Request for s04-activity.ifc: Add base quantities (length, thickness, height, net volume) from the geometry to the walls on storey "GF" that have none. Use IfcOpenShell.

First a look at what the model holds.

```python
import ifcopenshell
import ifcopenshell.util.element
import ifcopenshell.util.unit

model = ifcopenshell.open("s04-activity.ifc")
print(model.schema)
for unit_type in ("LENGTHUNIT", "AREAUNIT", "VOLUMEUNIT"):
    print(unit_type, ifcopenshell.util.unit.calculate_unit_scale(model, unit_type))
storey = next(s for s in model.by_type("IfcBuildingStorey") if s.Name == "GF")
walls = [e for e in ifcopenshell.util.element.get_decomposition(storey) if e.is_a("IfcWall")]
for e in sorted(walls, key=lambda e: e.id()):
    print(e.id(), e.is_a(), e.Name, list(ifcopenshell.util.element.get_psets(e, qtos_only=True)), sep=" | ")
```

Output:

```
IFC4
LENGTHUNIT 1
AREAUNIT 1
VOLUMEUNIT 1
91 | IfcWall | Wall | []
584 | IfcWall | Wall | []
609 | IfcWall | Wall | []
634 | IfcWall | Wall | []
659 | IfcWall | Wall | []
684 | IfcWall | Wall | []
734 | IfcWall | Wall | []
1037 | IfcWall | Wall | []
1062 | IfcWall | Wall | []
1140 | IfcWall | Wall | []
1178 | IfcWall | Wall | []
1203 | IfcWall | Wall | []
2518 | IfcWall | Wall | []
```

```python
import ifcopenshell
import ifcopenshell.api.pset
import ifcopenshell.geom
import ifcopenshell.util.element
import ifcopenshell.util.shape
import ifcopenshell.util.unit

model = ifcopenshell.open("s04-activity.ifc")
unit_scale = ifcopenshell.util.unit.calculate_unit_scale(model)
volume_scale = ifcopenshell.util.unit.calculate_unit_scale(model, "VOLUMEUNIT")
settings = ifcopenshell.geom.settings()

storey = next(s for s in model.by_type("IfcBuildingStorey") if s.Name == "GF")
walls = [e for e in ifcopenshell.util.element.get_decomposition(storey) if e.is_a("IfcWall")]

for e in sorted(walls, key=lambda e: e.id()):
    if ifcopenshell.util.element.get_psets(e, qtos_only=True, should_inherit=False):
        continue
    # Geometry comes back in metres, in the element's own axes.
    shape = ifcopenshell.geom.create_shape(settings, e)
    values = {
        "Length": ifcopenshell.util.shape.get_x(shape.geometry) / unit_scale,
        "Width": ifcopenshell.util.shape.get_y(shape.geometry) / unit_scale,
        "Height": ifcopenshell.util.shape.get_z(shape.geometry) / unit_scale,
        "NetVolume": ifcopenshell.util.shape.get_volume(shape.geometry) / volume_scale,
    }
    qto = ifcopenshell.api.pset.add_qto(model, product=e, name="Qto_WallBaseQuantities")
    ifcopenshell.api.pset.edit_qto(model, qto=qto, properties=values)
    print(e.id(), {k: round(v, 3) for k, v in values.items()})

model.write("s04-activity_updated.ifc")
```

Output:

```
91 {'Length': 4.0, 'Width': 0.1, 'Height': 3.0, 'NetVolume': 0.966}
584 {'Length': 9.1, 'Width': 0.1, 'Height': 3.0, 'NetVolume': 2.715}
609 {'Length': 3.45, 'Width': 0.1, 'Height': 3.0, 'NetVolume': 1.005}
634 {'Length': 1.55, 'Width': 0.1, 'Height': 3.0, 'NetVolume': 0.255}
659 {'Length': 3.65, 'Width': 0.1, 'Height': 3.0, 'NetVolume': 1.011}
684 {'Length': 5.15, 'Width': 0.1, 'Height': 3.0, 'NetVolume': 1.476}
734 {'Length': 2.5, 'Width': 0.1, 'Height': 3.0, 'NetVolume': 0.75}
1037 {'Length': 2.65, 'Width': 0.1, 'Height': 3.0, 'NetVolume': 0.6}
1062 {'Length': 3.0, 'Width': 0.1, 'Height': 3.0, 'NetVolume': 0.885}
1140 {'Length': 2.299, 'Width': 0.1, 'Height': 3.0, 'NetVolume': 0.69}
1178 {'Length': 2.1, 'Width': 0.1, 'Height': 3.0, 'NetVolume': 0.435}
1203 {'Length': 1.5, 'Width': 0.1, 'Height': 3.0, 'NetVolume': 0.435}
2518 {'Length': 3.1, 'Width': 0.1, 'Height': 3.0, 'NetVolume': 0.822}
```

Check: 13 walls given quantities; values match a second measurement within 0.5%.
